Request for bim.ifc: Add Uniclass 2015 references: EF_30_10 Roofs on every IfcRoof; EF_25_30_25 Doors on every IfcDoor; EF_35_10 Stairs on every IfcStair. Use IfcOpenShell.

First a look at what the model holds.

```python
import ifcopenshell

model = ifcopenshell.open("bim.ifc")
print(model.schema)
print("classifications:", [c.Name for c in model.by_type("IfcClassification")])
for ifc_class in ("IfcDoor", "IfcRoof", "IfcStair", "IfcWall", "IfcWindow"):
    print(ifc_class, len(model.by_type(ifc_class)))
```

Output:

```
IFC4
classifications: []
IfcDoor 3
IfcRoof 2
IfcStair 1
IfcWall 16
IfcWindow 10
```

```python
import ifcopenshell
import ifcopenshell.api.classification

model = ifcopenshell.open("bim.ifc")

system = ifcopenshell.api.classification.add_classification(model, classification="Uniclass 2015")

codes = {
    "IfcRoof": ("EF_30_10", "Roofs"),
    "IfcDoor": ("EF_25_30_25", "Doors"),
    "IfcStair": ("EF_35_10", "Stairs"),
}
for ifc_class, (code, name) in codes.items():
    products = model.by_type(ifc_class)
    ifcopenshell.api.classification.add_reference(
        model, products=products, classification=system, identification=code, name=name
    )
    print(code, len(products))

model.write("bim_edited.ifc")
```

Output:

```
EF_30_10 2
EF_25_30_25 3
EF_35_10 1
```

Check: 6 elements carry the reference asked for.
